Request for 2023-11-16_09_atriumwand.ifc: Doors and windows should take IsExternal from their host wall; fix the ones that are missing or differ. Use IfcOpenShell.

First a look at what the model holds.

```python
import ifcopenshell
import ifcopenshell.util.element

model = ifcopenshell.open("2023-11-16_09_atriumwand.ifc")
print(model.schema)
seen = {}
for e in model.by_type("IfcDoor") + model.by_type("IfcWindow"):
    if not e.FillsVoids:
        continue
    host = e.FillsVoids[0].RelatingOpeningElement.VoidsElements[0].RelatingBuildingElement
    own = ifcopenshell.util.element.get_pset(e, f"Pset_{e.is_a()[3:].removesuffix('StandardCase')}Common", "IsExternal")
    wall = ifcopenshell.util.element.get_pset(host, "Pset_WallCommon", "IsExternal")
    seen[e.is_a(), own, wall] = seen.get((e.is_a(), own, wall), 0) + 1
for (cls, own, wall), count in sorted(seen.items(), key=str):
    print(count, cls, "IsExternal:", own, "| host wall:", wall)
```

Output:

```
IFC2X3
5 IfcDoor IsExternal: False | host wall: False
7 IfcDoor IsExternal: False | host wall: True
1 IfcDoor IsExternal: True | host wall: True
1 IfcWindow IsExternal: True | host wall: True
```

```python
import ifcopenshell
import ifcopenshell.api.pset
import ifcopenshell.util.element

model = ifcopenshell.open("2023-11-16_09_atriumwand.ifc")

count = 0
for ifc_class, pset_name in (("IfcDoor", "Pset_DoorCommon"), ("IfcWindow", "Pset_WindowCommon")):
    for e in model.by_type(ifc_class):
        if not e.FillsVoids:
            continue
        host = e.FillsVoids[0].RelatingOpeningElement.VoidsElements[0].RelatingBuildingElement
        external = ifcopenshell.util.element.get_pset(host, "Pset_WallCommon", "IsExternal")
        if external is None or ifcopenshell.util.element.get_pset(e, pset_name, "IsExternal") == external:
            continue
        pset = ifcopenshell.api.pset.add_pset(model, product=e, name=pset_name)
        ifcopenshell.api.pset.edit_pset(model, pset=pset, properties={"IsExternal": external})
        count += 1

print(count, "updated")

model.write("2023-11-16_09_atriumwand_rev.ifc")
```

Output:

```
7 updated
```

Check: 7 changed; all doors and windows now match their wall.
